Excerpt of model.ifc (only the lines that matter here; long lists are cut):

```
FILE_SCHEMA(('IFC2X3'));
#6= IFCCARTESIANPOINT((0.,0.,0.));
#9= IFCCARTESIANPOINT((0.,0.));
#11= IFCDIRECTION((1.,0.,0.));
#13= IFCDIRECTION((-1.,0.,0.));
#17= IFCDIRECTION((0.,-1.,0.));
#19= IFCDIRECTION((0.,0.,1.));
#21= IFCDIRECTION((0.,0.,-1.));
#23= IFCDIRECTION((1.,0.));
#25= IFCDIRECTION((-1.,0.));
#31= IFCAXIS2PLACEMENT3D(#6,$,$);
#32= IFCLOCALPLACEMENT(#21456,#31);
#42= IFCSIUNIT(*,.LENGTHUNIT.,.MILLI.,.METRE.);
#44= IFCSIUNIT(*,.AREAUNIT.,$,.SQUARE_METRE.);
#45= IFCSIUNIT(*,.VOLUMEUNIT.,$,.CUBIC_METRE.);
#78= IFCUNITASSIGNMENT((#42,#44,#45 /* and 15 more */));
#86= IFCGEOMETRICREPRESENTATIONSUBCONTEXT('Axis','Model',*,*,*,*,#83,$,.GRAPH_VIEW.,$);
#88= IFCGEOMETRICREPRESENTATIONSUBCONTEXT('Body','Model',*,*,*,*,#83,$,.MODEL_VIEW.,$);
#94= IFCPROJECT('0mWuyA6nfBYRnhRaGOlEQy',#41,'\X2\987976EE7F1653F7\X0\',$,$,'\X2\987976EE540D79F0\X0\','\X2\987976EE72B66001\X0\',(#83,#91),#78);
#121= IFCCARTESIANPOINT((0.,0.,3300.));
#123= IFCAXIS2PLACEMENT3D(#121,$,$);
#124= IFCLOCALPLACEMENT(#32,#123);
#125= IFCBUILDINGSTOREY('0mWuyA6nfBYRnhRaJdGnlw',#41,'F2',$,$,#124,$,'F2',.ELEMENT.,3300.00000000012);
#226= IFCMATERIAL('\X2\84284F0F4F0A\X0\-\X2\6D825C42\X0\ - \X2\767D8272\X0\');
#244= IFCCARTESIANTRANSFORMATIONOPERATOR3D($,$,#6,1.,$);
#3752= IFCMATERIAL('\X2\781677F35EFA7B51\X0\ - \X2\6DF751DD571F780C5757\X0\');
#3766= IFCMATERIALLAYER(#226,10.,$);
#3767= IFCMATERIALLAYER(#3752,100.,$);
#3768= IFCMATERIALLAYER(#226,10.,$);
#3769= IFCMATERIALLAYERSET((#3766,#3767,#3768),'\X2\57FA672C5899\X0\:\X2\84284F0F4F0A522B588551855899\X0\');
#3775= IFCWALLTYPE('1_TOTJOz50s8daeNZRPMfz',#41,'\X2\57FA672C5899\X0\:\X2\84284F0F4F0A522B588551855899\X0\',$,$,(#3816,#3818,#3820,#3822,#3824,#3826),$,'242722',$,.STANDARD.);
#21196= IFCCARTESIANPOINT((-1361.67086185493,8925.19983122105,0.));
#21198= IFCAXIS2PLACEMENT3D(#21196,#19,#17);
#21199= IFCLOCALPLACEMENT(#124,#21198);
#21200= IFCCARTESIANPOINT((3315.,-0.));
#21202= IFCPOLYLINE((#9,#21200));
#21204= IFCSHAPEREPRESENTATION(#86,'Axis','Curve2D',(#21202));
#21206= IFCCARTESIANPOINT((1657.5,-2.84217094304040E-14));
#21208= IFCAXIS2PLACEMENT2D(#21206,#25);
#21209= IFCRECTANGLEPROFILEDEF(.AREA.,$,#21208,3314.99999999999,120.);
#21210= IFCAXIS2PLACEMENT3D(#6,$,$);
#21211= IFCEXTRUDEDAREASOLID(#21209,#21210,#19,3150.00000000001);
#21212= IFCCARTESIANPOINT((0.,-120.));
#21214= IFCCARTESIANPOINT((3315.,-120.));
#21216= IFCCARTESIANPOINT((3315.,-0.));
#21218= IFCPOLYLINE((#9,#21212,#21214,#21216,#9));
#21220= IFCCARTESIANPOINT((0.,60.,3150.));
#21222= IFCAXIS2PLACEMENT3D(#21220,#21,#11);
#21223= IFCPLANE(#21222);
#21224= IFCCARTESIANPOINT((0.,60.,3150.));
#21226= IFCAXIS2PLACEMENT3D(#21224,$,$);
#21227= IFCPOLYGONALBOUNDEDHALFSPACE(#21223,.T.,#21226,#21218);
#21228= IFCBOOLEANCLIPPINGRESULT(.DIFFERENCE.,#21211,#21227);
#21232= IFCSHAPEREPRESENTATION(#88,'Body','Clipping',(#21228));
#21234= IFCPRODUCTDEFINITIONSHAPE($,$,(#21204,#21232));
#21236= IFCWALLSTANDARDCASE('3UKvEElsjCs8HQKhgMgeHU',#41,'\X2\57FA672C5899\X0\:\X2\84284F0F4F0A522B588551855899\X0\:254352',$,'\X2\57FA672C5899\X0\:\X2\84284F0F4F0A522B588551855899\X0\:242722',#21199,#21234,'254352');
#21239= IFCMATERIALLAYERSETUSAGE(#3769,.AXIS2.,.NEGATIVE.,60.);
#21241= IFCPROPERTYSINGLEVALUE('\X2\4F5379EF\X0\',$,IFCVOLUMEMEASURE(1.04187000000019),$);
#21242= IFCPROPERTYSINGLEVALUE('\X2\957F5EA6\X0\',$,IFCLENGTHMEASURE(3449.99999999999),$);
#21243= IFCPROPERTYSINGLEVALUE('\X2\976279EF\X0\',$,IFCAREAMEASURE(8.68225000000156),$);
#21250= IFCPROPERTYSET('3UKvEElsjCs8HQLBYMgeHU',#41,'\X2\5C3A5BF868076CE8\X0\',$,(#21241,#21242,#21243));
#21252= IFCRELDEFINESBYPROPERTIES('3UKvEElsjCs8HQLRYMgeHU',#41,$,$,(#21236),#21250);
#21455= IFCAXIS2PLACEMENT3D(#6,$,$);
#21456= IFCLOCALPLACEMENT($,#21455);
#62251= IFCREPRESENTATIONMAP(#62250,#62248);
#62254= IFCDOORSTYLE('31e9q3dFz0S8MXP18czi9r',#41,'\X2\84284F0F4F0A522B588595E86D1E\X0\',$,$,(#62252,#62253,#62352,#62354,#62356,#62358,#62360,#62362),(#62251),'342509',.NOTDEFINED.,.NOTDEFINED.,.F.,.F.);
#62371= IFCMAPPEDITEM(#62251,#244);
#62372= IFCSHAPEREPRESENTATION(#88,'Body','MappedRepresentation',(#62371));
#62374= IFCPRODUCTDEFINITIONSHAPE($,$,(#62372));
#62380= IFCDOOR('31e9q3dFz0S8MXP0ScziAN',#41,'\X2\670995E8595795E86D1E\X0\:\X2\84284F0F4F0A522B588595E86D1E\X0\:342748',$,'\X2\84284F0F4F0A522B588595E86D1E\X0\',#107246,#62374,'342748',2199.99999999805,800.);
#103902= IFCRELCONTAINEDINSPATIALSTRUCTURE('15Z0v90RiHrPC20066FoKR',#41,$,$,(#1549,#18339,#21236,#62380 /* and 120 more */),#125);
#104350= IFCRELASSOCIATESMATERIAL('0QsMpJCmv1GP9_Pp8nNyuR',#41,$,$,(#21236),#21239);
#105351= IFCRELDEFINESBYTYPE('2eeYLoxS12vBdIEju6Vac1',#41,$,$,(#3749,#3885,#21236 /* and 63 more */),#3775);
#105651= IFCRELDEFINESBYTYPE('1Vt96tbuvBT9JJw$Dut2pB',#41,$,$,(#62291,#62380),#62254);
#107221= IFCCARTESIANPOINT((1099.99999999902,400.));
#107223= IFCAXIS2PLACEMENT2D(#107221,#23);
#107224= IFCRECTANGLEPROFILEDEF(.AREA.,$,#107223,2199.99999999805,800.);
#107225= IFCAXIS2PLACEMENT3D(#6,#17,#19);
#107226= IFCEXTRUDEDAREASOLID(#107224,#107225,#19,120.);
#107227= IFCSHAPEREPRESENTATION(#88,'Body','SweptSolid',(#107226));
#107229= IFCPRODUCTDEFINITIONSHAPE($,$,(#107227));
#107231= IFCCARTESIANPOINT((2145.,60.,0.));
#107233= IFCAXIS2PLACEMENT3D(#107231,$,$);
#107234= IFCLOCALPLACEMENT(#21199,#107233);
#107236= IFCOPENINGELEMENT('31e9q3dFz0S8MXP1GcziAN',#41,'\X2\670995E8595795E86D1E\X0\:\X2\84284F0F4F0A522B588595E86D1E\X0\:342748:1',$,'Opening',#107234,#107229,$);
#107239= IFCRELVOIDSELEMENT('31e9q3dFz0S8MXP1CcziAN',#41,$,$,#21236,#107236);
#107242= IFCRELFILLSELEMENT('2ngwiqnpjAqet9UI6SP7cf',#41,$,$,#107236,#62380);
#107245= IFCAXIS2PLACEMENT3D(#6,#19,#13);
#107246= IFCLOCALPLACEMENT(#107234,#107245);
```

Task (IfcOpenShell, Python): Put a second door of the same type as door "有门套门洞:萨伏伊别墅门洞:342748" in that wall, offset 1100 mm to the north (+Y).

```python
import ifcopenshell
import ifcopenshell.api.feature
import ifcopenshell.api.geometry
import ifcopenshell.api.pset
import ifcopenshell.api.root
import ifcopenshell.geom
import ifcopenshell.util.element
import ifcopenshell.util.placement
import ifcopenshell.util.shape
import ifcopenshell.util.unit

model = ifcopenshell.open("model.ifc")
unit_scale = ifcopenshell.util.unit.calculate_unit_scale(model)
area_scale = ifcopenshell.util.unit.calculate_unit_scale(model, "AREAUNIT")
volume_scale = ifcopenshell.util.unit.calculate_unit_scale(model, "VOLUMEUNIT")
settings = ifcopenshell.geom.settings()


def volume(element):
    """Net volume in cubic metres, openings subtracted."""
    shape = ifcopenshell.geom.create_shape(settings, element)
    return ifcopenshell.util.shape.get_volume(shape.geometry)


def reuse_history(source, copy):
    """copy_class also copies each property set's owner history, people and application; keep the originals."""
    for rel in copy.IsDefinedBy:
        if rel.is_a("IfcRelDefinesByProperties") and (history := rel.RelatingPropertyDefinition.OwnerHistory):
            rel.RelatingPropertyDefinition.OwnerHistory = source.OwnerHistory
            ifcopenshell.util.element.remove_deep2(model, history)


door = model.by_guid("31e9q3dFz0S8MXP0ScziAN")
opening = door.FillsVoids[0].RelatingOpeningElement
wall = opening.VoidsElements[0].RelatingBuildingElement
before = volume(wall)
shift = ifcopenshell.util.placement.get_local_placement(wall.ObjectPlacement)[:3, 0] * -1.1 / unit_scale

# copy_class copies the void relationship, type, container and properties, but no geometry.
new_opening = ifcopenshell.api.root.copy_class(model, product=opening)
new_opening.Representation = ifcopenshell.util.element.copy_deep(
    model, opening.Representation, exclude=["IfcGeometricRepresentationContext", "IfcRepresentationMap"]
)
new_opening.Name = "有门套门洞:萨伏伊别墅门洞"
new_door = ifcopenshell.api.root.copy_class(model, product=door)
new_door.Representation = ifcopenshell.util.element.copy_deep(
    model, door.Representation, exclude=["IfcGeometricRepresentationContext", "IfcRepresentationMap"]
)
new_door.Name = "有门套门洞:萨伏伊别墅门洞"
new_door.Tag = None
reuse_history(door, new_door)
fills = ifcopenshell.api.feature.add_filling(model, opening=new_opening, element=new_door)
fills.OwnerHistory = new_door.OwnerHistory  # required in IFC2X3

for old, new in ((opening, new_opening), (door, new_door)):
    matrix = ifcopenshell.util.placement.get_local_placement(old.ObjectPlacement)
    matrix[:3, 3] += shift
    ifcopenshell.api.geometry.edit_object_placement(model, product=new, matrix=matrix, is_si=False)

after = volume(wall)
thickness = 0.12  # wall thickness in metres

# Update the wall's stored quantities.
pset = model.by_id(ifcopenshell.util.element.get_pset(wall, "尺寸标注", should_inherit=False)["id"])
ifcopenshell.api.pset.edit_pset(model, pset=pset, properties={
    "体积": model.create_entity("IfcVolumeMeasure", after / volume_scale),
    "面积": model.create_entity("IfcAreaMeasure", after / thickness / area_scale),
})

print(f"wall volume {before:.3f} -> {after:.3f} m3")

model.write("model_rev.ifc")
```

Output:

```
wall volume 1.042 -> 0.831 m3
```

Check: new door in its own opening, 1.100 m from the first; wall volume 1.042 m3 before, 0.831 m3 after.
